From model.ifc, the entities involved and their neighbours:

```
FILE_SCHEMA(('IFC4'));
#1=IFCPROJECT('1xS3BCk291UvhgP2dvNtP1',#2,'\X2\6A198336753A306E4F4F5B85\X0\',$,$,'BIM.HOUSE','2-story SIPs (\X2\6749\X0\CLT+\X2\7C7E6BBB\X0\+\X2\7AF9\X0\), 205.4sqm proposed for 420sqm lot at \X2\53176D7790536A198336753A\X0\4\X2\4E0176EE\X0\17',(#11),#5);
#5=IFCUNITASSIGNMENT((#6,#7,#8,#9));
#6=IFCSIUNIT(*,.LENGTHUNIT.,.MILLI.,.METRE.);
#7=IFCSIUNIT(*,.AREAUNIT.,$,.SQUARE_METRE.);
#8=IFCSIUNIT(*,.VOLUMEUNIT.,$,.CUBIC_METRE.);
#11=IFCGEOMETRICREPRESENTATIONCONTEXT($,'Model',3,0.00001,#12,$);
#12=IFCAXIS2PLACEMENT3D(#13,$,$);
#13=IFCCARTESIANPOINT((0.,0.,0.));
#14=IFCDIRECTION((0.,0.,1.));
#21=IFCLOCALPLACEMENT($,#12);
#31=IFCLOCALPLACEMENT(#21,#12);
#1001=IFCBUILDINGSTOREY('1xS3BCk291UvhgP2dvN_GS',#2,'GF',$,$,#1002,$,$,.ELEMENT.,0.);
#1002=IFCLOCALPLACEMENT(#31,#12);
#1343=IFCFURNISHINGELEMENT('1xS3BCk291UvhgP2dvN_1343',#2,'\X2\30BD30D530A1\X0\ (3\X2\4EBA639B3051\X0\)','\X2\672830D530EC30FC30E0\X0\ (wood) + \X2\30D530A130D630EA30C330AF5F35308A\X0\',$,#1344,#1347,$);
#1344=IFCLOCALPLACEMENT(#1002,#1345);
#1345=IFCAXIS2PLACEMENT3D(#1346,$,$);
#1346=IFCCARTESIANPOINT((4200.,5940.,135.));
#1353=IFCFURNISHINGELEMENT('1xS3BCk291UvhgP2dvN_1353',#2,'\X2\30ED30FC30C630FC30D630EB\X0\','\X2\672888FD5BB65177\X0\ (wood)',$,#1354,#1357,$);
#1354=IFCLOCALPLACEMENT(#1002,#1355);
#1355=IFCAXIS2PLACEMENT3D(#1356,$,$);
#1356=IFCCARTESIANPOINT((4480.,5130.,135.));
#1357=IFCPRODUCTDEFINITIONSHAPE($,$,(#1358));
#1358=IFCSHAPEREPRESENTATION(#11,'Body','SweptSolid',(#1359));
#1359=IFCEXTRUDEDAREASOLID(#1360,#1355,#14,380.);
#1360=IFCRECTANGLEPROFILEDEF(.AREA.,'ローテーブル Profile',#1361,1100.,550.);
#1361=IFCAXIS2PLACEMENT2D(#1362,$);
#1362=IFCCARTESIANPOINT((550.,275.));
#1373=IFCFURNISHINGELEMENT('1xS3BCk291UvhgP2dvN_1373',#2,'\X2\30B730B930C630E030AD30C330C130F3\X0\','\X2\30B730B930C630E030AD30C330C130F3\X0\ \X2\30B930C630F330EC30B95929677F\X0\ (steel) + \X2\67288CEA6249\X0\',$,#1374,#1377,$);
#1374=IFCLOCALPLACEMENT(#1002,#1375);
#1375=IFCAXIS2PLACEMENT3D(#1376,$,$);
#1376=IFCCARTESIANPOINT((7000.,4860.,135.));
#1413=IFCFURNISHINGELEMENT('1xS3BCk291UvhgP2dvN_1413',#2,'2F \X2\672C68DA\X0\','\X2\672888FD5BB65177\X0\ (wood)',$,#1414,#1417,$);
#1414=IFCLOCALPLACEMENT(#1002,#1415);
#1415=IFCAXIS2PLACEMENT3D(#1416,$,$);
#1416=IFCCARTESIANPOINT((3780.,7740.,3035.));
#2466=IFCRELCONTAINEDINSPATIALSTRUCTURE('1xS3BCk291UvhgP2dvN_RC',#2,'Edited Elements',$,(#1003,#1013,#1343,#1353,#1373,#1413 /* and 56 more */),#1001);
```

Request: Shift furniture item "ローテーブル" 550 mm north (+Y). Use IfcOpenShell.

```python
import ifcopenshell
import ifcopenshell.api.geometry
import ifcopenshell.util.placement
import ifcopenshell.util.unit

model = ifcopenshell.open("model.ifc")
unit_scale = ifcopenshell.util.unit.calculate_unit_scale(model)

item = model.by_guid("1xS3BCk291UvhgP2dvN_1353")
matrix = ifcopenshell.util.placement.get_local_placement(item.ObjectPlacement)
matrix[1, 3] += 0.55 / unit_scale
ifcopenshell.api.geometry.edit_object_placement(model, product=item, matrix=matrix, is_si=False)

print(ifcopenshell.util.placement.get_local_placement(item.ObjectPlacement).round(3) + 0.0)

model.write("model_edited.ifc")
```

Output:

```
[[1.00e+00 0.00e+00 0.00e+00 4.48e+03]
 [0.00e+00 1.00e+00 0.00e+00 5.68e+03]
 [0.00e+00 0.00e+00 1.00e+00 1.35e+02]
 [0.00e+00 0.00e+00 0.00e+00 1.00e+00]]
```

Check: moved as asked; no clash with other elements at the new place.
